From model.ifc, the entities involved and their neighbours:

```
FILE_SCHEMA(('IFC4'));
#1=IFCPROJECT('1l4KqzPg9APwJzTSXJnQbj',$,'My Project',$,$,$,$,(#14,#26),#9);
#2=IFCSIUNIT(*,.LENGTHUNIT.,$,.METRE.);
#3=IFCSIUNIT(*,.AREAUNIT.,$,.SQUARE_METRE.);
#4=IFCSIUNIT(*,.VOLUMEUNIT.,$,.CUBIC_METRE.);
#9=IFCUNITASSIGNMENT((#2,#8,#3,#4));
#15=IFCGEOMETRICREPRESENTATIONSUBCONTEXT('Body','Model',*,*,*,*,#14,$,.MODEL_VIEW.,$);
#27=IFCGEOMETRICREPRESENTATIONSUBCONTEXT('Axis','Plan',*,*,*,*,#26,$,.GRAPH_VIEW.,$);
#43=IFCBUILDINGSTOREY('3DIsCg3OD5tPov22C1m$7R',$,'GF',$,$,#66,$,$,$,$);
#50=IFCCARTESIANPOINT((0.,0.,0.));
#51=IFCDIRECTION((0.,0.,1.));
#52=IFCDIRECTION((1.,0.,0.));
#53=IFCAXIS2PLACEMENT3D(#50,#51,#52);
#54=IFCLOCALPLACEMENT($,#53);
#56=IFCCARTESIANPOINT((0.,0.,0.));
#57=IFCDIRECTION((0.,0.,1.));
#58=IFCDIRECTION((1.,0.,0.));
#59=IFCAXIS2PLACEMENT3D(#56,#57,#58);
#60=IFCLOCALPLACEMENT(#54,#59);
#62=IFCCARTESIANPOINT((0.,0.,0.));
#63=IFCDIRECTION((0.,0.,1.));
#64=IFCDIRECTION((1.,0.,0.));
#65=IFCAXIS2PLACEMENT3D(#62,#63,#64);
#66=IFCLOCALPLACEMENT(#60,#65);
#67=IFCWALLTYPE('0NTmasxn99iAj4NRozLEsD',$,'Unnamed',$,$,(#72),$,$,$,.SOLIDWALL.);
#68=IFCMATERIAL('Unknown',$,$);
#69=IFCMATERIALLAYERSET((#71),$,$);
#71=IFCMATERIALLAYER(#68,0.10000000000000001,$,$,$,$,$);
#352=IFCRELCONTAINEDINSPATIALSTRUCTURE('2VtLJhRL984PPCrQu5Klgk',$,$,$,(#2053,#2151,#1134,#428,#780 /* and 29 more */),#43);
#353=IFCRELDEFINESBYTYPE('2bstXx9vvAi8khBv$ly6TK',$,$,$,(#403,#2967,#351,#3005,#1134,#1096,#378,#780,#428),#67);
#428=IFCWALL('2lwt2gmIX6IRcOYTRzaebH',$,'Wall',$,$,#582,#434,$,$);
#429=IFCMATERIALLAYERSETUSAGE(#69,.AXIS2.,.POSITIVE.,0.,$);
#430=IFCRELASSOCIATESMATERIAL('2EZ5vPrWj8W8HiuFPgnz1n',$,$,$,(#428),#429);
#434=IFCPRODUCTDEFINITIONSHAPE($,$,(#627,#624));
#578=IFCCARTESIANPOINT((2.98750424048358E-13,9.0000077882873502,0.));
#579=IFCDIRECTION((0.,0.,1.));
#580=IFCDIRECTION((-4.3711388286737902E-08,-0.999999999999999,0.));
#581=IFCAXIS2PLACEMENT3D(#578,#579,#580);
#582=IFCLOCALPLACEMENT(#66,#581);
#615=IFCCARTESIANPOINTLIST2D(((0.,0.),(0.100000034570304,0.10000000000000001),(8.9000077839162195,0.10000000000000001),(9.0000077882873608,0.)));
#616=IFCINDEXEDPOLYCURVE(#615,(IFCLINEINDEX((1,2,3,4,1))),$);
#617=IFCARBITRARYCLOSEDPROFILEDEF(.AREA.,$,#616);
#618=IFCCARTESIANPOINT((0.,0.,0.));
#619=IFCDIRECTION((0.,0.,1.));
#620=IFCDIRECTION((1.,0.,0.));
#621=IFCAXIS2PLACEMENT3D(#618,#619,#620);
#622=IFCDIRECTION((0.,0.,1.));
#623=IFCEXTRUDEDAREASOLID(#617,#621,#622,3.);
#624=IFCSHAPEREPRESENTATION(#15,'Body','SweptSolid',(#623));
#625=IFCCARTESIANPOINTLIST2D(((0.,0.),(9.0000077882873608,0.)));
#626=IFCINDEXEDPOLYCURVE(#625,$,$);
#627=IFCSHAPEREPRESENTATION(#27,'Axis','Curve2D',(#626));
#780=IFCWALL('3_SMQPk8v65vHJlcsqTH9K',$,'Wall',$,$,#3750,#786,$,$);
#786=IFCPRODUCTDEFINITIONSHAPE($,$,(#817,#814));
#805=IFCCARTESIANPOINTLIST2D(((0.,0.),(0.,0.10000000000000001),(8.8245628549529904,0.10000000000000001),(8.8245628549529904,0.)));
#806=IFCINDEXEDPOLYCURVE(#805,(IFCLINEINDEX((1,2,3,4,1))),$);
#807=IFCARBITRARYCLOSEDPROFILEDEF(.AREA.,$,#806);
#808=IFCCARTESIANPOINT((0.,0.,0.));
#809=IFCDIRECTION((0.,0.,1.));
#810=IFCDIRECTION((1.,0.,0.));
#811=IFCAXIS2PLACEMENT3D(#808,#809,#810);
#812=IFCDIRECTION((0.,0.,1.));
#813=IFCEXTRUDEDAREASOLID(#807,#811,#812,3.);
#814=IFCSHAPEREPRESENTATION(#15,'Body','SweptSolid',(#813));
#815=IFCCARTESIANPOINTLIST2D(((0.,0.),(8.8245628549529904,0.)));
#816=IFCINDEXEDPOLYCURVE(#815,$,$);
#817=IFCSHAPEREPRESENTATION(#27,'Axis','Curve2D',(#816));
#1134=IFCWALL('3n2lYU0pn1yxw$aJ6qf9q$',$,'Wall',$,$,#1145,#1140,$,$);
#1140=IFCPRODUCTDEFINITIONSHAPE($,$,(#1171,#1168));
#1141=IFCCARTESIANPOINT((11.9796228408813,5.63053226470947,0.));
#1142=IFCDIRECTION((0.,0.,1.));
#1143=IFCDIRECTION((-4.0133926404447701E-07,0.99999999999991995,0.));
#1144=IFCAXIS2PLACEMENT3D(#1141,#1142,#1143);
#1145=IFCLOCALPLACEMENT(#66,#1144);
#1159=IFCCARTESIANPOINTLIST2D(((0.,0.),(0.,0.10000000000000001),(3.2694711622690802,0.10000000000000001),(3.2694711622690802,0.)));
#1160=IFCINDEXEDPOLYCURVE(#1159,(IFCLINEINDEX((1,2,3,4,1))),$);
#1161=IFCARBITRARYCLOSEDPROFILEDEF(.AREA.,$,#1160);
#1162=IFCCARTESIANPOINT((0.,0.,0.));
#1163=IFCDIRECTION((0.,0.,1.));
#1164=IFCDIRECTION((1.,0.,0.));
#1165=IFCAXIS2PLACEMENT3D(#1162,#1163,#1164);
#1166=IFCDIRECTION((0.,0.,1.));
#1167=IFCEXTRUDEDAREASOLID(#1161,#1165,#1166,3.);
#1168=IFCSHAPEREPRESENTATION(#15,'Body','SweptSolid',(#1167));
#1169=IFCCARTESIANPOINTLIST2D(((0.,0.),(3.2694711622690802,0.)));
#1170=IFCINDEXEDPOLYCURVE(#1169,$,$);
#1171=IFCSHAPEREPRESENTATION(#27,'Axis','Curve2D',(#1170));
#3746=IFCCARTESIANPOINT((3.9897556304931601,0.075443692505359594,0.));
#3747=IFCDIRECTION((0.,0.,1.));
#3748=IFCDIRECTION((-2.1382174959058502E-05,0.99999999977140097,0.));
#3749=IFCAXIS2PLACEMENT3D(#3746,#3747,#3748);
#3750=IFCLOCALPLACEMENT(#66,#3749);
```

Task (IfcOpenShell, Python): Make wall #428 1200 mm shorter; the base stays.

```python
import ifcopenshell
import ifcopenshell.geom
import ifcopenshell.util.representation
import ifcopenshell.util.shape

model = ifcopenshell.open("model.ifc")
settings = ifcopenshell.geom.settings()


def volume(element):
    """Net volume in cubic metres, openings subtracted."""
    shape = ifcopenshell.geom.create_shape(settings, element)
    return ifcopenshell.util.shape.get_volume(shape.geometry)


wall = model.by_guid("2lwt2gmIX6IRcOYTRzaebH")
before = volume(wall)

body = ifcopenshell.util.representation.get_representation(wall, "Model", "Body")
solid = body.Items[0]
old_height = solid.Depth
solid.Depth -= 1.2
after = volume(wall)

print(f"height {old_height:g} -> {solid.Depth:g}, volume {before:.3f} -> {after:.3f} m3")

model.write("model_v2.ifc")
```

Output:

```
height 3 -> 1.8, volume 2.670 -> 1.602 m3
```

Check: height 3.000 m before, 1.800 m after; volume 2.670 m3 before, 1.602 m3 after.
